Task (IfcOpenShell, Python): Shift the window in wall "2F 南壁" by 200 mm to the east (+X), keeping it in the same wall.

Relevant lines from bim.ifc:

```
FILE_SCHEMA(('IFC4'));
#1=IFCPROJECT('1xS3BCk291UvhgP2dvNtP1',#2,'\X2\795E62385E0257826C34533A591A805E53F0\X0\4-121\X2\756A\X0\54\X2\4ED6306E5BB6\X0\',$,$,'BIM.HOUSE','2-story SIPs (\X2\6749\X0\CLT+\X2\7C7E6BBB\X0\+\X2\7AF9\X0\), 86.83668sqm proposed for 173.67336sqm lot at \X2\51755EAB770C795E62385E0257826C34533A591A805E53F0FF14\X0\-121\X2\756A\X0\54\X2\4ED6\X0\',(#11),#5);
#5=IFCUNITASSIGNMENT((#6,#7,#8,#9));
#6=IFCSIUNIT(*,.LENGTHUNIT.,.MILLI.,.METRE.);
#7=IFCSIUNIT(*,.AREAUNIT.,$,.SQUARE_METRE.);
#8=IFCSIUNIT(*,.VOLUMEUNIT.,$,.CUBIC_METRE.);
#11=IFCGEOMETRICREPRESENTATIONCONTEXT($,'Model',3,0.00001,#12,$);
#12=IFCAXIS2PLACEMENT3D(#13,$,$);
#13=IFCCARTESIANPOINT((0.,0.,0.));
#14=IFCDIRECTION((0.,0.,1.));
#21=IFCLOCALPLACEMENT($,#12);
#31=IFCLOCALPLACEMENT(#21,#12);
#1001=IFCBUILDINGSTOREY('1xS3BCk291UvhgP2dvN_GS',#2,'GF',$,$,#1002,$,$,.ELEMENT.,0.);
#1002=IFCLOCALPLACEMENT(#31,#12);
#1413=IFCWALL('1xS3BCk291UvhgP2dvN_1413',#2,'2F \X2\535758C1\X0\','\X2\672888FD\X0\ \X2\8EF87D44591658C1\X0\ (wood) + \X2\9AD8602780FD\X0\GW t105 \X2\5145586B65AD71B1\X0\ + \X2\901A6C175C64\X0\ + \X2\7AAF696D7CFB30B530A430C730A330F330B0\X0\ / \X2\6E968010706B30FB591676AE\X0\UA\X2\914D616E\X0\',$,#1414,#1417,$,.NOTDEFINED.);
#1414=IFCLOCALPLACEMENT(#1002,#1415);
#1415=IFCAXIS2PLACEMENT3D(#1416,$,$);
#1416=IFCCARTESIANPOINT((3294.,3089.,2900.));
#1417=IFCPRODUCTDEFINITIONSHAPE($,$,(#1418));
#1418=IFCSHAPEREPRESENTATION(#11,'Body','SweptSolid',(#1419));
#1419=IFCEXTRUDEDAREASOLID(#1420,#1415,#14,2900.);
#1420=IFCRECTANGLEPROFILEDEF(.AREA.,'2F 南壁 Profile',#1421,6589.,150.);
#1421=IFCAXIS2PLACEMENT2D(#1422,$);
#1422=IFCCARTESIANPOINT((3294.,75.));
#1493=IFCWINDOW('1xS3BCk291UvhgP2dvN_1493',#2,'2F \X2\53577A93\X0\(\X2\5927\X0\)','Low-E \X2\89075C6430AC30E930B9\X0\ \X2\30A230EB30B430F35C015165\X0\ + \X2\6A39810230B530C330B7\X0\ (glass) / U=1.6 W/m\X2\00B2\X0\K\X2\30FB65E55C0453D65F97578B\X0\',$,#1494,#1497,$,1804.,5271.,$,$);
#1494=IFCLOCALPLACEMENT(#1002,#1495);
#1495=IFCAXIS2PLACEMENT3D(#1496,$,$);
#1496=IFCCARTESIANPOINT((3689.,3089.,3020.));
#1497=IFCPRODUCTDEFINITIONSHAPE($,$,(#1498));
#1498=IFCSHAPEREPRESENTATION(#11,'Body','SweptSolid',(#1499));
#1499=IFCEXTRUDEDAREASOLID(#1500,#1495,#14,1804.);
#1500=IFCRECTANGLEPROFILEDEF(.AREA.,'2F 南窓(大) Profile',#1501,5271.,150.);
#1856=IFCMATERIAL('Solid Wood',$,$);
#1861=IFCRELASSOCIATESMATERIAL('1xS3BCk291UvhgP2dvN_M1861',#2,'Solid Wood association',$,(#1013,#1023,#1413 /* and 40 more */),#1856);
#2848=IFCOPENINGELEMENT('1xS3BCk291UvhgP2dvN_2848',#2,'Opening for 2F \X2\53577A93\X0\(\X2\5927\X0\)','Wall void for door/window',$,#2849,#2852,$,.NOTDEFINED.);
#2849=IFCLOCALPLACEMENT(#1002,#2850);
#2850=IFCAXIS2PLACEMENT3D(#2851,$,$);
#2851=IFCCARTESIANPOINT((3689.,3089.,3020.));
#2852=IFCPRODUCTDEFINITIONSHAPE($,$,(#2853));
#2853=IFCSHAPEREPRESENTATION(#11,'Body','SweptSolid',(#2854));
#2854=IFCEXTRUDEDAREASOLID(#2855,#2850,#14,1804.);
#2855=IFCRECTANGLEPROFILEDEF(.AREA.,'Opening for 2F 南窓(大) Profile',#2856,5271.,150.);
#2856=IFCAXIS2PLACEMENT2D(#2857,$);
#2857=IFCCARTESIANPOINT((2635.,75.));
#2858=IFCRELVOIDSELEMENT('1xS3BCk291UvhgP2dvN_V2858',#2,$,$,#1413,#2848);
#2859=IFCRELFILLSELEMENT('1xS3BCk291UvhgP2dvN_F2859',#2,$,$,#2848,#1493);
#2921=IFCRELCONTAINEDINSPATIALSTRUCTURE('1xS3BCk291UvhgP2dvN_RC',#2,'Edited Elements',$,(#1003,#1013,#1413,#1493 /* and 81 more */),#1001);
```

```python
import ifcopenshell
import ifcopenshell.api.geometry
import ifcopenshell.util.placement
import ifcopenshell.util.unit

model = ifcopenshell.open("bim.ifc")
unit_scale = ifcopenshell.util.unit.calculate_unit_scale(model)

window = model.by_guid("1xS3BCk291UvhgP2dvN_1493")
opening = window.FillsVoids[0].RelatingOpeningElement
wall = opening.VoidsElements[0].RelatingBuildingElement

wall_matrix = ifcopenshell.util.placement.get_local_placement(wall.ObjectPlacement)
shift = wall_matrix[:3, 0] * 0.2 / unit_scale
before = ifcopenshell.util.placement.get_local_placement(window.ObjectPlacement)[:3, 3].copy()

# The window is not placed relative to its opening, so move both.
for product in (opening, window):
    matrix = ifcopenshell.util.placement.get_local_placement(product.ObjectPlacement)
    matrix[:3, 3] += shift
    ifcopenshell.api.geometry.edit_object_placement(model, product=product, matrix=matrix, is_si=False)

after = ifcopenshell.util.placement.get_local_placement(window.ObjectPlacement)[:3, 3]
print("window moved by", (after - before).round(3) + 0.0)

model.write("bim_updated.ifc")
```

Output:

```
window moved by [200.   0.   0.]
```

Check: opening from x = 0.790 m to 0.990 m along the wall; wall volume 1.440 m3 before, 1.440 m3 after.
